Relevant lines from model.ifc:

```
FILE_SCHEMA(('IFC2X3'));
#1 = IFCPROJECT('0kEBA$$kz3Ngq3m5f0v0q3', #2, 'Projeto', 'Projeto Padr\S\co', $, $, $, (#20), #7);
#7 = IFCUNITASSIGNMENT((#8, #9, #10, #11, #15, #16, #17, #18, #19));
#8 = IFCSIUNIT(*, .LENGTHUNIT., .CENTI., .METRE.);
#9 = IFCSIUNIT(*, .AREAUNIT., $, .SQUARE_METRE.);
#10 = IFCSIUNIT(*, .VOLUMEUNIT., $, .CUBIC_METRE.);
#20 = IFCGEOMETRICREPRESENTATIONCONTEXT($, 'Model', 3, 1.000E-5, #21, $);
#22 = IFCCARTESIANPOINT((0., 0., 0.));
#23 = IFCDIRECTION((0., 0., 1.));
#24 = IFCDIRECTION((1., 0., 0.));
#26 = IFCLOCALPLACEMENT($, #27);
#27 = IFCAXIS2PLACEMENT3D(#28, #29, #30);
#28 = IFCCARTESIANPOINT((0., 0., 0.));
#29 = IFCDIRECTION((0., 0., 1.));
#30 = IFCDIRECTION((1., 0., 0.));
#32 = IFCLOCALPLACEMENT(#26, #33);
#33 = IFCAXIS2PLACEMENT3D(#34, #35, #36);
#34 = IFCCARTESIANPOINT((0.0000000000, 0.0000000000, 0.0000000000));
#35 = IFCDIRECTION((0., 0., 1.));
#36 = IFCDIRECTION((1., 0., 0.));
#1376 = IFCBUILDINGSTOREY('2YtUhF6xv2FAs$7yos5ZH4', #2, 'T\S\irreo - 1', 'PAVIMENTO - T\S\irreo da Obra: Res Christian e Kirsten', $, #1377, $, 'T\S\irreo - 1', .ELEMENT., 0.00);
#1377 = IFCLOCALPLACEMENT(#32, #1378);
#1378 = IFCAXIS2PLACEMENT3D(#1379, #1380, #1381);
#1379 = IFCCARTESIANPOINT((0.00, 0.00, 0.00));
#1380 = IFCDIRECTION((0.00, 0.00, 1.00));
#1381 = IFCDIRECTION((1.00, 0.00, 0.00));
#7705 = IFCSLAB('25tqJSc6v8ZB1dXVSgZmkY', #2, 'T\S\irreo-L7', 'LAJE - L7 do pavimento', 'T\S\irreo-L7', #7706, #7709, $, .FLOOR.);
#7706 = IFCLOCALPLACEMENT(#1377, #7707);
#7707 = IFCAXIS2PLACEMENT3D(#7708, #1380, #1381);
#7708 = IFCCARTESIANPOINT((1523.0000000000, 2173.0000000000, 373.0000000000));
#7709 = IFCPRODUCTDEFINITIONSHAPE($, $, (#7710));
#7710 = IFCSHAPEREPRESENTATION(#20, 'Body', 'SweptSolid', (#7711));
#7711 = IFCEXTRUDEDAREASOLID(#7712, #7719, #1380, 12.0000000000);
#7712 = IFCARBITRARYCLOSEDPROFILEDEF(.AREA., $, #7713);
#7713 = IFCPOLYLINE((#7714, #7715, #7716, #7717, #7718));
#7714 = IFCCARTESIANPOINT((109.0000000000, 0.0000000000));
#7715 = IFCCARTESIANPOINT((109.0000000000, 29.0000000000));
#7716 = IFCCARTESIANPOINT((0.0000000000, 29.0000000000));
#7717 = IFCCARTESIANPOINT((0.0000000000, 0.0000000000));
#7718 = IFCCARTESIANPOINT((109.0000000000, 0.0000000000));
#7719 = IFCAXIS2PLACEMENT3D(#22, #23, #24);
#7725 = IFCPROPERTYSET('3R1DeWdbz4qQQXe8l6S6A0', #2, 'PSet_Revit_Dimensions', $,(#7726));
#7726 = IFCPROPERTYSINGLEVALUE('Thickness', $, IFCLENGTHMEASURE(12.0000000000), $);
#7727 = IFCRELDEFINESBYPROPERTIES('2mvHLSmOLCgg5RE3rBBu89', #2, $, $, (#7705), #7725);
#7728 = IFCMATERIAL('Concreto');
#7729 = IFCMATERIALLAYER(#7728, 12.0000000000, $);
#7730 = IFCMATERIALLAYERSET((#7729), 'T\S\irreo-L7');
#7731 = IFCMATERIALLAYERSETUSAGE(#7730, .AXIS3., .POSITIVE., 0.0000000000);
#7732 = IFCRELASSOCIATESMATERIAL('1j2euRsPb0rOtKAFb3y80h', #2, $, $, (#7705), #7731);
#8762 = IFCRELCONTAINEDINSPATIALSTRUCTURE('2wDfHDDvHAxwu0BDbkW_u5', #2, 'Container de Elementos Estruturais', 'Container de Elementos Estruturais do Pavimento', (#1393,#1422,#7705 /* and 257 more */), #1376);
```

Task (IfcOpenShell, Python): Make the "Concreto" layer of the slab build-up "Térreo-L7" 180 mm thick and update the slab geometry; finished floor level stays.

```python
import ifcopenshell
import ifcopenshell.api.pset
import ifcopenshell.util.element
import ifcopenshell.util.unit

model = ifcopenshell.open("model.ifc")
unit_scale = ifcopenshell.util.unit.calculate_unit_scale(model)

layer_set = model.by_id(7730)
layer = next(l for l in layer_set.MaterialLayers if l.Material and l.Material.Name == "Concreto")
change = 0.18 / unit_scale - layer.LayerThickness
layer.LayerThickness += change

# Geometry does not follow the layer set by itself.
slabs = [e for e in ifcopenshell.util.element.get_elements_by_material(model, layer_set) if e.is_a("IfcSlab")]
for slab in sorted(slabs, key=lambda e: e.id()):
    body = next(r for r in slab.Representation.Representations if r.RepresentationIdentifier == "Body")
    solid = body.Items[0]
    old_depth = solid.Depth
    solid.Depth += change
    # Extruded upwards: lower the start of the extrusion so the top stays.
    x, y, z = solid.Position.Location.Coordinates
    solid.Position.Location = model.createIfcCartesianPoint((x, y, z - change))
    pset = model.by_id(ifcopenshell.util.element.get_pset(slab, "PSet_Revit_Dimensions", should_inherit=False)["id"])
    ifcopenshell.api.pset.edit_pset(model, pset=pset, properties={
        "Thickness": model.create_entity("IfcLengthMeasure", solid.Depth),
    })
    print(slab.id(), f"{old_depth:g} -> {solid.Depth:g}")

# The layers are counted up from the underside, which has moved.
for usage in {ifcopenshell.util.element.get_material(slab) for slab in slabs}:
    usage.OffsetFromReferenceLine -= change

model.write("model-out.ifc")
```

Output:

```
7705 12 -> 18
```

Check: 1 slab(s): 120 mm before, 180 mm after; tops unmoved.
